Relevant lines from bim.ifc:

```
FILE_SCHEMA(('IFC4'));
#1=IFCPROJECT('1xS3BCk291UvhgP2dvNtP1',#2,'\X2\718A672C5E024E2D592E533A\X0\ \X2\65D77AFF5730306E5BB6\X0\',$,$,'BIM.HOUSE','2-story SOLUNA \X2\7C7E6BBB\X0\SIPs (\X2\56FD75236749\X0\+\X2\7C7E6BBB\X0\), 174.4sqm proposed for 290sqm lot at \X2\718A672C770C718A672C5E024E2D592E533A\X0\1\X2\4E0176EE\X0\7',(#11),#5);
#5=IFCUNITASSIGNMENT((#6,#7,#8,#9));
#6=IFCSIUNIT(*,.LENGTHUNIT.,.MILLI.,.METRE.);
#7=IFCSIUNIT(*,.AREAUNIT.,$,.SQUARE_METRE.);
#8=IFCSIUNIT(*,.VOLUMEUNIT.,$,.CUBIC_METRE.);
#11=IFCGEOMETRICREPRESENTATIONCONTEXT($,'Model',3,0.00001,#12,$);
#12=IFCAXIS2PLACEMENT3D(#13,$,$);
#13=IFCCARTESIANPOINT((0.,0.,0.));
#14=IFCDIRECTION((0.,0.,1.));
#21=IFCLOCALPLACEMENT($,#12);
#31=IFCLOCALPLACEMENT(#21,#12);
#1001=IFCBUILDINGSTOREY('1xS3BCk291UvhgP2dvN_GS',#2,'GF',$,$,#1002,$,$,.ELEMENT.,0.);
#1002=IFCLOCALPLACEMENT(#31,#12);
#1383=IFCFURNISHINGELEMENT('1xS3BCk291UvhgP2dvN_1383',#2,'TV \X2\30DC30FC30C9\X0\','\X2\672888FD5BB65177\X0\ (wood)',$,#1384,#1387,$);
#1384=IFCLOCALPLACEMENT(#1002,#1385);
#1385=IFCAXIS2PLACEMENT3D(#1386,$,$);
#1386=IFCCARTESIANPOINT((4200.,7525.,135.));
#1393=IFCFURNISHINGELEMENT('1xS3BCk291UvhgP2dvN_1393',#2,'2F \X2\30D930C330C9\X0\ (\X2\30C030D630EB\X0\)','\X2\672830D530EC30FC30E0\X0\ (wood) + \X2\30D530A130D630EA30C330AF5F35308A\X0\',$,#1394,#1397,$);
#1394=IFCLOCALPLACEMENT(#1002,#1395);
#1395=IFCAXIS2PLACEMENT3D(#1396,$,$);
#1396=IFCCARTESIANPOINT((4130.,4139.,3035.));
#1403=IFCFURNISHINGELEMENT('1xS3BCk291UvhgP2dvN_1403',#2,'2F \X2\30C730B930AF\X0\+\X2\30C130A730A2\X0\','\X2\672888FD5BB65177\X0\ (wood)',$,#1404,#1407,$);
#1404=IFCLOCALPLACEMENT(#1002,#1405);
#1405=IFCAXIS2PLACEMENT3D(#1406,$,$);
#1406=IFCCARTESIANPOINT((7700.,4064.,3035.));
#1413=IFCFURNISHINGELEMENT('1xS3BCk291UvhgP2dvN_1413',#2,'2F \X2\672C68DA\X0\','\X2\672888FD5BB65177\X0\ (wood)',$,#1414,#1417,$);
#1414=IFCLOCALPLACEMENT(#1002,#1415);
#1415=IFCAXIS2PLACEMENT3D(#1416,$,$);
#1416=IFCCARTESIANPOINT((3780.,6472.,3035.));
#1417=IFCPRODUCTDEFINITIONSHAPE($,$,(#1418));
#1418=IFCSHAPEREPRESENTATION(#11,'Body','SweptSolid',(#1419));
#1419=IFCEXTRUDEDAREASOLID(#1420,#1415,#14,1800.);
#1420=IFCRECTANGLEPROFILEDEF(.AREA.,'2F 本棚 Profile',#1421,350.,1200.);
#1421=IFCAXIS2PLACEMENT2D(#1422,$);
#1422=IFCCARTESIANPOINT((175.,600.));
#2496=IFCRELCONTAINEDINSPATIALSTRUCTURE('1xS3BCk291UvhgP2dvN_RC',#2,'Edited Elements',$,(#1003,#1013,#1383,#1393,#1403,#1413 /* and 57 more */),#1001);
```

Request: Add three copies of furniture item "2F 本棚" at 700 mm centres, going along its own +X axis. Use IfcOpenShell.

```python
import ifcopenshell
import ifcopenshell.api.geometry
import ifcopenshell.api.root
import ifcopenshell.util.element
import ifcopenshell.util.placement
import ifcopenshell.util.unit

model = ifcopenshell.open("bim.ifc")
unit_scale = ifcopenshell.util.unit.calculate_unit_scale(model)


def reuse_history(source, copy):
    """copy_class also copies each property set's owner history, people and application; keep the originals."""
    for rel in copy.IsDefinedBy:
        if rel.is_a("IfcRelDefinesByProperties") and (history := rel.RelatingPropertyDefinition.OwnerHistory):
            rel.RelatingPropertyDefinition.OwnerHistory = source.OwnerHistory
            ifcopenshell.util.element.remove_deep2(model, history)


source = model.by_guid("1xS3BCk291UvhgP2dvN_1413")
base = ifcopenshell.util.placement.get_local_placement(source.ObjectPlacement)
step = base[:3, 0] * 0.7 / unit_scale

for i in range(1, 4):
    copy = ifcopenshell.api.root.copy_class(model, product=source)
    copy.Representation = ifcopenshell.util.element.copy_deep(
        model, source.Representation, exclude=["IfcGeometricRepresentationContext", "IfcRepresentationMap"]
    )
    reuse_history(source, copy)
    matrix = base.copy()
    matrix[:3, 3] += i * step
    print("added at", matrix[:3, 3].round(3) + 0.0)
    ifcopenshell.api.geometry.edit_object_placement(model, product=copy, matrix=matrix, is_si=False)

model.write("bim_updated.ifc")
```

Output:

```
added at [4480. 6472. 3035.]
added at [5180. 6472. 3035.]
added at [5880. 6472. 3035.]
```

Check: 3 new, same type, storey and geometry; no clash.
